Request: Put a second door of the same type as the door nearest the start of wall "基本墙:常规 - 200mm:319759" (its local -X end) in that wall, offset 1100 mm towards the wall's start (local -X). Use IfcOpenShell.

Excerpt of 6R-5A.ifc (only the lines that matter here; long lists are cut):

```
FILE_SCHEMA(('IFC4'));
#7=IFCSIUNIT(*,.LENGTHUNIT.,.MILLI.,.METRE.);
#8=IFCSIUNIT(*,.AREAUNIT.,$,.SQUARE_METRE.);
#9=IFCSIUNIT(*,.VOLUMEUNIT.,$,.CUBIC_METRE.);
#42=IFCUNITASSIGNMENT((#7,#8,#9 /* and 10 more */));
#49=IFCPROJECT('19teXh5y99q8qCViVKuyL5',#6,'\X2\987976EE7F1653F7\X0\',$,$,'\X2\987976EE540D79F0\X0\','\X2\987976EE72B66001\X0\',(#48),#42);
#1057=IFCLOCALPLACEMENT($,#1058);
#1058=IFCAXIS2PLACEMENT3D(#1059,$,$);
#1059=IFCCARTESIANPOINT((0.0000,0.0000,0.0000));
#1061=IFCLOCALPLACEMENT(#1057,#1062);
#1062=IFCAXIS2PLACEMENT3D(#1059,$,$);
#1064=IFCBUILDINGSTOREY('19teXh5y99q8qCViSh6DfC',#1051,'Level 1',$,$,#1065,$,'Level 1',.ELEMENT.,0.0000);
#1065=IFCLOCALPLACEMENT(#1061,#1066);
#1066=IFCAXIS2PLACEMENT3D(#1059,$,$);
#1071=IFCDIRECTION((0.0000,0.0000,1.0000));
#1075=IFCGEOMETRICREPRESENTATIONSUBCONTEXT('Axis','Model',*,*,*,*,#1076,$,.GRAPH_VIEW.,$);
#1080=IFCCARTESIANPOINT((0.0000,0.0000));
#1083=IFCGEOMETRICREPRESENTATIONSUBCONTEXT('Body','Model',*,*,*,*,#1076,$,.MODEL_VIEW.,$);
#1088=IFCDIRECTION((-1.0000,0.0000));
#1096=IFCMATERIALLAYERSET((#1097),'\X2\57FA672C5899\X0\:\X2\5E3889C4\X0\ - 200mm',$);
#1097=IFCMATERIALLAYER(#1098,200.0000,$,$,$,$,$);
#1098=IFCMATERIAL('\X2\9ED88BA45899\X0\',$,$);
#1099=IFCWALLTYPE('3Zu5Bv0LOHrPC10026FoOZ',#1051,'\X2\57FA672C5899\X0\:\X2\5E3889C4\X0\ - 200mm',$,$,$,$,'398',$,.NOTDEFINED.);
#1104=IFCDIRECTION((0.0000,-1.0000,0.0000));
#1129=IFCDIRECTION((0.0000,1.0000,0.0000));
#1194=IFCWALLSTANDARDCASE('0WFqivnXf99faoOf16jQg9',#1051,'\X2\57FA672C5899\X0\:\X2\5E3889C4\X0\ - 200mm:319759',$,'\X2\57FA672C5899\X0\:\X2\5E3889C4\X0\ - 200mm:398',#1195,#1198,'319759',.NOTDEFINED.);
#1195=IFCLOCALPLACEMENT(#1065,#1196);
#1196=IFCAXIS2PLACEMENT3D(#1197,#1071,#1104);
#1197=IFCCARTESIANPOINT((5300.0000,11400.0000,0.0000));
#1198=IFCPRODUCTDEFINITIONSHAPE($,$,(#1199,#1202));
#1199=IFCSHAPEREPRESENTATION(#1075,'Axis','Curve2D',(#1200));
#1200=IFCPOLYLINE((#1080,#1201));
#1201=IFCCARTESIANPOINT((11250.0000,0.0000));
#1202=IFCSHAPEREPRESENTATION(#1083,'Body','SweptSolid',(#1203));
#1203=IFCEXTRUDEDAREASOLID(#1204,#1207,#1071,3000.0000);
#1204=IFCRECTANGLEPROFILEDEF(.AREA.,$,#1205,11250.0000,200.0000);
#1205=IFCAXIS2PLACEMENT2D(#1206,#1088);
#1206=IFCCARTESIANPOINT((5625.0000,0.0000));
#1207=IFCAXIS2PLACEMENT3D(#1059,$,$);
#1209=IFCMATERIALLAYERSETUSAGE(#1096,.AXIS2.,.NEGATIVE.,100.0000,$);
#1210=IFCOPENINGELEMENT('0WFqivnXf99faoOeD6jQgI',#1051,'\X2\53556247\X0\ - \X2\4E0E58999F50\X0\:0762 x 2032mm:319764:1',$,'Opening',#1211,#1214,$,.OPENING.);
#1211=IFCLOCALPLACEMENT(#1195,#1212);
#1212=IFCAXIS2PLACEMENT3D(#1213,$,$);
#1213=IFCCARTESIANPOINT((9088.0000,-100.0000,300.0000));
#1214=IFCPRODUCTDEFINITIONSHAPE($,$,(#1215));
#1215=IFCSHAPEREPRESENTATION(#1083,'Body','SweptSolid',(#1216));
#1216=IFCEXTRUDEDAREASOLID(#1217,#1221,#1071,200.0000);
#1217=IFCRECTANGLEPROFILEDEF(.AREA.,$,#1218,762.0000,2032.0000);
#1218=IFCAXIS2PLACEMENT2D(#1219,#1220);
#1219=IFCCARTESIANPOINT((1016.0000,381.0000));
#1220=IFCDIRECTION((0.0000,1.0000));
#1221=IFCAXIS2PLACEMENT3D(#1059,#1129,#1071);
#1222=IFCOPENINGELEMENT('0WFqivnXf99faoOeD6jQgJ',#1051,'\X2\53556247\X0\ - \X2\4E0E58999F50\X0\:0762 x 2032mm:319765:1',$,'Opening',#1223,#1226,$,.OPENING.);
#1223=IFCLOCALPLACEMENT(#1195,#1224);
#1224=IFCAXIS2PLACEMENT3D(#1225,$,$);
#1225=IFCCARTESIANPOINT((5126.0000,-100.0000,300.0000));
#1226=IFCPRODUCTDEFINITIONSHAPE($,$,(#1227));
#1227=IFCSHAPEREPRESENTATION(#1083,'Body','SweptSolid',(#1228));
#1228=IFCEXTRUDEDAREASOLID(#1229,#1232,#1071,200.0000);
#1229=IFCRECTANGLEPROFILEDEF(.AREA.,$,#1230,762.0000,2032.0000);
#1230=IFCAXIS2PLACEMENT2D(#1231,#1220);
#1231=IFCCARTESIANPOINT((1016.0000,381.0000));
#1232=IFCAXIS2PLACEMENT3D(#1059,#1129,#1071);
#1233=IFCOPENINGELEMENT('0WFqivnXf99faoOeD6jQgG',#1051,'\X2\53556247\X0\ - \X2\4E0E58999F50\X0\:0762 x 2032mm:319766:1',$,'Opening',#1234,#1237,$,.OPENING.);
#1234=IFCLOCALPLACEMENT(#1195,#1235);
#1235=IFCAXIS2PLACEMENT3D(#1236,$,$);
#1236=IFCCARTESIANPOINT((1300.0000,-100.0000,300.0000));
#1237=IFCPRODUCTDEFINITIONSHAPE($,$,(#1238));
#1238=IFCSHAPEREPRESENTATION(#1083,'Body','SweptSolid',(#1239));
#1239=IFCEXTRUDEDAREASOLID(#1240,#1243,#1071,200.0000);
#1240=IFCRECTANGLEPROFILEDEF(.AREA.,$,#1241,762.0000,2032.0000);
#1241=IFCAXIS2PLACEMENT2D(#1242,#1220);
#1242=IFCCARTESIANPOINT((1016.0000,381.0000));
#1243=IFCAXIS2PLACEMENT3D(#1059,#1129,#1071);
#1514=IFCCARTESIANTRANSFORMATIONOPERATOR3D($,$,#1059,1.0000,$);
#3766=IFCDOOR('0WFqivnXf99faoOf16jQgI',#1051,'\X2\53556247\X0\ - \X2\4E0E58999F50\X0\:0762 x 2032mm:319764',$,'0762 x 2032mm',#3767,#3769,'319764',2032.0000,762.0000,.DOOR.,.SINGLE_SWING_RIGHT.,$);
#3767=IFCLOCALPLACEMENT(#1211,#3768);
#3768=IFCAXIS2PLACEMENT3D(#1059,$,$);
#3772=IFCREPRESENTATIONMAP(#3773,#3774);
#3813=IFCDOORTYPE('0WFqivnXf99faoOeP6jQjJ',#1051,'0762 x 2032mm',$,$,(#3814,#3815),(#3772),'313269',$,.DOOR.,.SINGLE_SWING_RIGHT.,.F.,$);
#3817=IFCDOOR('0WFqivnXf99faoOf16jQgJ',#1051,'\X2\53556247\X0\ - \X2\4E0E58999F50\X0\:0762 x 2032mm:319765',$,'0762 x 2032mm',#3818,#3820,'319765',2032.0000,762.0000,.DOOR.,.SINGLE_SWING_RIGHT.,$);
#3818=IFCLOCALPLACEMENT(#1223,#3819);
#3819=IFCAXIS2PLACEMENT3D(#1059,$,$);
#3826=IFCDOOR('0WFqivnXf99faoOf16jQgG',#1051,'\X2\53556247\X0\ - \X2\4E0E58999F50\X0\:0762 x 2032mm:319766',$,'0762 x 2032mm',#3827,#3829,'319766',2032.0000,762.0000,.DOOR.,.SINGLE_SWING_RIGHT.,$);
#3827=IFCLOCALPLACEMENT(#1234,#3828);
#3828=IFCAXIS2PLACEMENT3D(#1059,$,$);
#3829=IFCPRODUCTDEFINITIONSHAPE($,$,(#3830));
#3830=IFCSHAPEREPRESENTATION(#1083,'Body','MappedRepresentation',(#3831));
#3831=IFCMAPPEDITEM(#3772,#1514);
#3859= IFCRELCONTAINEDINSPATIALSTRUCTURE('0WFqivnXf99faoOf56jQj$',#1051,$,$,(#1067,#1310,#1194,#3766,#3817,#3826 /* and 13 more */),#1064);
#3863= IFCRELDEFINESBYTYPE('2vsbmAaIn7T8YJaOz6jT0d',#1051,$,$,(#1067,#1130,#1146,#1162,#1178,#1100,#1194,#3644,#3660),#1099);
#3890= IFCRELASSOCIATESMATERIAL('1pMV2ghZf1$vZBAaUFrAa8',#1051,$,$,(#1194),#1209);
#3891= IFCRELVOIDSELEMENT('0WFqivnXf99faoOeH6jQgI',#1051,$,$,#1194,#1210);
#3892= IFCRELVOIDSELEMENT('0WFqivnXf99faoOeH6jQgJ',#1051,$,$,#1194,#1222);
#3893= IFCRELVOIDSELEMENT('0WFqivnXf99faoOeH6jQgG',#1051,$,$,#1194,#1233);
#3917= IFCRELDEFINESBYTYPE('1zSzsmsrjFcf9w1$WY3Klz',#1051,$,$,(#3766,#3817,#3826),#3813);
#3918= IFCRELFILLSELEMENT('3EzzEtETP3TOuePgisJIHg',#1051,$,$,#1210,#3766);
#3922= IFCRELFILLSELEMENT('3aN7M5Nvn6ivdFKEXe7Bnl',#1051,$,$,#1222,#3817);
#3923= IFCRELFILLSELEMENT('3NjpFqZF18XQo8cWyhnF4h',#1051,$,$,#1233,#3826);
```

```python
import ifcopenshell
import ifcopenshell.api.feature
import ifcopenshell.api.geometry
import ifcopenshell.api.root
import ifcopenshell.geom
import ifcopenshell.util.element
import ifcopenshell.util.placement
import ifcopenshell.util.shape

model = ifcopenshell.open("6R-5A.ifc")
settings = ifcopenshell.geom.settings()


def volume(element):
    """Net volume in cubic metres, openings subtracted."""
    shape = ifcopenshell.geom.create_shape(settings, element)
    return ifcopenshell.util.shape.get_volume(shape.geometry)


def reuse_history(source, copy):
    """copy_class also copies each property set's owner history, people and application; keep the originals."""
    for rel in copy.IsDefinedBy:
        if rel.is_a("IfcRelDefinesByProperties") and (history := rel.RelatingPropertyDefinition.OwnerHistory):
            rel.RelatingPropertyDefinition.OwnerHistory = source.OwnerHistory
            ifcopenshell.util.element.remove_deep2(model, history)


door = model.by_guid("0WFqivnXf99faoOf16jQgG")
opening = door.FillsVoids[0].RelatingOpeningElement
wall = opening.VoidsElements[0].RelatingBuildingElement
before = volume(wall)
shift = ifcopenshell.util.placement.get_local_placement(wall.ObjectPlacement)[:3, 0] * -1100.0

# copy_class copies the void relationship, type, container and properties, but no geometry.
new_opening = ifcopenshell.api.root.copy_class(model, product=opening)
new_opening.Representation = ifcopenshell.util.element.copy_deep(
    model, opening.Representation, exclude=["IfcGeometricRepresentationContext", "IfcRepresentationMap"]
)
new_opening.Name = "单扇 - 与墙齐:0762 x 2032mm"
new_door = ifcopenshell.api.root.copy_class(model, product=door)
new_door.Representation = ifcopenshell.util.element.copy_deep(
    model, door.Representation, exclude=["IfcGeometricRepresentationContext", "IfcRepresentationMap"]
)
new_door.Name = "单扇 - 与墙齐:0762 x 2032mm"
new_door.Tag = None
reuse_history(door, new_door)
ifcopenshell.api.feature.add_filling(model, opening=new_opening, element=new_door)

for old, new in ((opening, new_opening), (door, new_door)):
    matrix = ifcopenshell.util.placement.get_local_placement(old.ObjectPlacement)
    matrix[:3, 3] += shift
    ifcopenshell.api.geometry.edit_object_placement(model, product=new, matrix=matrix, is_si=False)

after = volume(wall)

print(f"wall volume {before:.3f} -> {after:.3f} m3")

model.write("6R-5A_v2.ifc")
```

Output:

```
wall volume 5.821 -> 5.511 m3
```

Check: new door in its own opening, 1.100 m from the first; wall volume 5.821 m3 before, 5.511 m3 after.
